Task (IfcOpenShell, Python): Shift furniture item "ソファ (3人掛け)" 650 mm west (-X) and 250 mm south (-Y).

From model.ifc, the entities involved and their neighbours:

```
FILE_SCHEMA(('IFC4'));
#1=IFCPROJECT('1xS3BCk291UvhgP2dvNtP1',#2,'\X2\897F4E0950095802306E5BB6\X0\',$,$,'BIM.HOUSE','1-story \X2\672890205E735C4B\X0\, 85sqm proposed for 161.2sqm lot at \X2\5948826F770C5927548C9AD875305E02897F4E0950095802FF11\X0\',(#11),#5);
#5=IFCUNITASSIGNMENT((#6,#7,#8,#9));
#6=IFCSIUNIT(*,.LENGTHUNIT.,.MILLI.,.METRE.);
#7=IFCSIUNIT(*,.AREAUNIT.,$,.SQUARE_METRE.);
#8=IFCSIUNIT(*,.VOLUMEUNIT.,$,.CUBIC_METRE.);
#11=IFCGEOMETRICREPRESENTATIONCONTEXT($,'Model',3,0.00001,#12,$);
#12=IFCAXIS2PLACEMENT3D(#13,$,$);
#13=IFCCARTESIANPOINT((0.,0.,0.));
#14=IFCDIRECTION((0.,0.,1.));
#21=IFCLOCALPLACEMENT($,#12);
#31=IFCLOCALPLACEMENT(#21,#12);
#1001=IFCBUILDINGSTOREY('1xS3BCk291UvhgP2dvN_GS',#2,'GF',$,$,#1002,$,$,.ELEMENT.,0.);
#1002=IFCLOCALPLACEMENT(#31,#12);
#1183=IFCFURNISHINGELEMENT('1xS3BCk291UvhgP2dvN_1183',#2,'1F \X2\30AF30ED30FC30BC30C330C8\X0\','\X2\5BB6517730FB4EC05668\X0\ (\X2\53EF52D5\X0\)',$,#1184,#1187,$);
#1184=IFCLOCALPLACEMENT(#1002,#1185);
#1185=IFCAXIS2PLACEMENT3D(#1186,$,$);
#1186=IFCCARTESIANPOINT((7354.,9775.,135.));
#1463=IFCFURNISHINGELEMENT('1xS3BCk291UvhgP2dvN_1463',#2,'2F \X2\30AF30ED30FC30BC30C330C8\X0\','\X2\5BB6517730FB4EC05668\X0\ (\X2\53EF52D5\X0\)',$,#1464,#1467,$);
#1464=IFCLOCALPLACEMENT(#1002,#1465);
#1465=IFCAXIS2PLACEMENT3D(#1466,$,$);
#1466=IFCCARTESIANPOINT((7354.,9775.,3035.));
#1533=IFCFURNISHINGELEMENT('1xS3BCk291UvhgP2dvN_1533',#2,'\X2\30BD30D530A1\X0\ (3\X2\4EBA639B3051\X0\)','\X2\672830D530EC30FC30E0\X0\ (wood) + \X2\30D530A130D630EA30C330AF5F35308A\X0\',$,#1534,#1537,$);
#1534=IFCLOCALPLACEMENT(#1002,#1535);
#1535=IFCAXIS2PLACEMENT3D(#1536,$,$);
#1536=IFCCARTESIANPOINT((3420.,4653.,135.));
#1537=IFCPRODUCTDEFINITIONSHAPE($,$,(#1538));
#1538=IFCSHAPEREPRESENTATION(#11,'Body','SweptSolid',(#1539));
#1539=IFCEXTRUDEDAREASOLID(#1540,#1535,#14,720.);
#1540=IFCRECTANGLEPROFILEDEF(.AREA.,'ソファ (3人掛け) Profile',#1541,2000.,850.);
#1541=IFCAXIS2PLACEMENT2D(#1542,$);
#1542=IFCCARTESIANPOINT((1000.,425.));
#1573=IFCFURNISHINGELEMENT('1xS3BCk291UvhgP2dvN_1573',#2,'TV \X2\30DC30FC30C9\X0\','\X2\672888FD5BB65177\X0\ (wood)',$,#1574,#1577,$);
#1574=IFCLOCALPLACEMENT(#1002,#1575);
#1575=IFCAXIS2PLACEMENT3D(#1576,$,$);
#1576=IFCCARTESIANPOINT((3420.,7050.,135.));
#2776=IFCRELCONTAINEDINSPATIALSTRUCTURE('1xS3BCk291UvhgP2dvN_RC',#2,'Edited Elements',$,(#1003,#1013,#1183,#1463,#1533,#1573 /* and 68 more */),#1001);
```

```python
import ifcopenshell
import ifcopenshell.api.geometry
import ifcopenshell.util.placement
import ifcopenshell.util.unit

model = ifcopenshell.open("model.ifc")
unit_scale = ifcopenshell.util.unit.calculate_unit_scale(model)

item = model.by_guid("1xS3BCk291UvhgP2dvN_1533")
matrix = ifcopenshell.util.placement.get_local_placement(item.ObjectPlacement)
matrix[0, 3] -= 0.65 / unit_scale
matrix[1, 3] -= 0.25 / unit_scale
ifcopenshell.api.geometry.edit_object_placement(model, product=item, matrix=matrix, is_si=False)

print(ifcopenshell.util.placement.get_local_placement(item.ObjectPlacement).round(3) + 0.0)

model.write("model_rev.ifc")
```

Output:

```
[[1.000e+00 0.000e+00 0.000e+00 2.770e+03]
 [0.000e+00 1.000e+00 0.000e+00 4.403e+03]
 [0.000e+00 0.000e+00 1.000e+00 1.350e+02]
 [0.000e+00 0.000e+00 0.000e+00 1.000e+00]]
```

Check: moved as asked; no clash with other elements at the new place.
